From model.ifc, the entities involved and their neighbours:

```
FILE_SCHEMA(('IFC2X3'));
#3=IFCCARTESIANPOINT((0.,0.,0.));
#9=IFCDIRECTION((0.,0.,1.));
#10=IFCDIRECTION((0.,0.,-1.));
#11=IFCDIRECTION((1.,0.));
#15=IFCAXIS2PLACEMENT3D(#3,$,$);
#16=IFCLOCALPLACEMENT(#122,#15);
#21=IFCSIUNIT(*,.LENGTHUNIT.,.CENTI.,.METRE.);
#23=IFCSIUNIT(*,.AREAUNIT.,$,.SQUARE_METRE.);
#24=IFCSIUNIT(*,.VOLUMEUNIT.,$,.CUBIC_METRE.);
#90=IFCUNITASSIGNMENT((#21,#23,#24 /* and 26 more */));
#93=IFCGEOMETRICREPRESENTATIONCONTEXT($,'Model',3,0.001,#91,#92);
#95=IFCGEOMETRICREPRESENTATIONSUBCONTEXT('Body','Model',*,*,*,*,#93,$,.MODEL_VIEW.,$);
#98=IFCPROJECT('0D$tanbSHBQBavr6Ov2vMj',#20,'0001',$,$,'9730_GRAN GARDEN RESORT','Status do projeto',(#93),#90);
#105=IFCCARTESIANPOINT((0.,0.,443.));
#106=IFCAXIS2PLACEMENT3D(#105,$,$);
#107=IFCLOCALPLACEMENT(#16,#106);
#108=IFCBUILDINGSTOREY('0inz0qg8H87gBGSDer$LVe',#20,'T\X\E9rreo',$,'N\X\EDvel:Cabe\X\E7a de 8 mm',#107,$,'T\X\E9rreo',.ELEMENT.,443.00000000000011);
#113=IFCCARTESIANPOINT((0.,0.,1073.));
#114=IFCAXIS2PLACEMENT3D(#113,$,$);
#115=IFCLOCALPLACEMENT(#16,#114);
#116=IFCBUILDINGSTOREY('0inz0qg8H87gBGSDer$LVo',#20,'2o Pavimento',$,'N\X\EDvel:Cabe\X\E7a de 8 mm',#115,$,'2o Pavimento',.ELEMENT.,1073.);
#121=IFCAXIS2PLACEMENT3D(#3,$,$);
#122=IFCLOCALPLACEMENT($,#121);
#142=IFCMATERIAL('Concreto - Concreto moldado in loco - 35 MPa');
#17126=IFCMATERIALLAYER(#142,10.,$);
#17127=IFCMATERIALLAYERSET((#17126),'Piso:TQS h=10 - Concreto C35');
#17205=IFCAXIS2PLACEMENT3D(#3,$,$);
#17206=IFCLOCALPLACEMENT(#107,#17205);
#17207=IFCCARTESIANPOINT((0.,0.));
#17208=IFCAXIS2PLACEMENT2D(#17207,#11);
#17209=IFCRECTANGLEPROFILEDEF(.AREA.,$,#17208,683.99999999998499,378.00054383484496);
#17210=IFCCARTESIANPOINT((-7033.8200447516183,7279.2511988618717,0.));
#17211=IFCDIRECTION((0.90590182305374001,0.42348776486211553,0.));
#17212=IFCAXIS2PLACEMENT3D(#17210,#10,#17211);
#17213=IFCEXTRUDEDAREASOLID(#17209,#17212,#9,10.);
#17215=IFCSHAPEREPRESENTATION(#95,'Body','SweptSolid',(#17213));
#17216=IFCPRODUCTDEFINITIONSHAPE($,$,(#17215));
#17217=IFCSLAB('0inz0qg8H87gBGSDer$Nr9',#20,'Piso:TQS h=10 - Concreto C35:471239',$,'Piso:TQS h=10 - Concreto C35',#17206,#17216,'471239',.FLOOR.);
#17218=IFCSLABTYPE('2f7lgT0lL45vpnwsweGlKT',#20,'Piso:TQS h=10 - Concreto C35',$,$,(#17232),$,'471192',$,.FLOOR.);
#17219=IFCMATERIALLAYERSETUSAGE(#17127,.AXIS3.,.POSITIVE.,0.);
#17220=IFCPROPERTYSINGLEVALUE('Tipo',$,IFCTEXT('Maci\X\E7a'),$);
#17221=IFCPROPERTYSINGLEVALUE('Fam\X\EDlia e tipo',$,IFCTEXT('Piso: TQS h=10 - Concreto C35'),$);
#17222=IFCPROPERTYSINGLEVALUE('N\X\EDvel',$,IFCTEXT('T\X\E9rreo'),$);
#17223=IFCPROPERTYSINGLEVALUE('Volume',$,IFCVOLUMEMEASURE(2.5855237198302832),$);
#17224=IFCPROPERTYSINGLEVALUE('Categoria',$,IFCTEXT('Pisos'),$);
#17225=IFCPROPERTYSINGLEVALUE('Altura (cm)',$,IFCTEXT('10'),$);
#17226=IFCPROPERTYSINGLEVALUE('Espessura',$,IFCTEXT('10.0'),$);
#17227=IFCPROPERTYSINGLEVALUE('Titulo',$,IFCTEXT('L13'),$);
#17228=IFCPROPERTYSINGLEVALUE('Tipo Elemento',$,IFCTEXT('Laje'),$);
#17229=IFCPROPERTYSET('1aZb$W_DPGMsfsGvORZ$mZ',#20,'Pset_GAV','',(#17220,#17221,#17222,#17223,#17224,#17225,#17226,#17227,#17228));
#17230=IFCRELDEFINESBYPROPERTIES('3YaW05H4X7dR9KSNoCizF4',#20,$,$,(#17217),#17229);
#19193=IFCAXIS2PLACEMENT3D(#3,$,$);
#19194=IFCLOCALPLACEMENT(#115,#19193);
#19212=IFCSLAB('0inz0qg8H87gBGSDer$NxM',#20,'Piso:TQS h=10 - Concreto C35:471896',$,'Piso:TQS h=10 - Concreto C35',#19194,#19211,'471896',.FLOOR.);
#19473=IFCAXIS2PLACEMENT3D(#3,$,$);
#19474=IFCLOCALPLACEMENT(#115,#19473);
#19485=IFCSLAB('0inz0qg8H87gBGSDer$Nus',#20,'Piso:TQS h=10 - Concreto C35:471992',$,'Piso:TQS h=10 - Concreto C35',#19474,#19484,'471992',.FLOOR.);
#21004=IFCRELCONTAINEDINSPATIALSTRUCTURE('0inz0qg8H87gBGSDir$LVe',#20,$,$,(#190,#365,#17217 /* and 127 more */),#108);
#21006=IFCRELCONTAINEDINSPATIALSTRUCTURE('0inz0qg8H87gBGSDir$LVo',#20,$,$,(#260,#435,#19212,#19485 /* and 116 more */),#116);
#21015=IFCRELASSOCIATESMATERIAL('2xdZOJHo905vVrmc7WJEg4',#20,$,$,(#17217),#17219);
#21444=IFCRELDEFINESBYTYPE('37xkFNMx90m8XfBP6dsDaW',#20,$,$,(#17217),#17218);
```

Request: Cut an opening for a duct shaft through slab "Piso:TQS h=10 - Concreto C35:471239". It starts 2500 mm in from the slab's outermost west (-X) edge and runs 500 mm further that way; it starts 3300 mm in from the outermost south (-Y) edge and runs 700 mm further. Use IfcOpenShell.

```python
import numpy as np
import ifcopenshell
import ifcopenshell.api.feature
import ifcopenshell.api.geometry
import ifcopenshell.api.pset
import ifcopenshell.api.root
import ifcopenshell.geom
import ifcopenshell.util.element
import ifcopenshell.util.placement
import ifcopenshell.util.representation
import ifcopenshell.util.shape
import ifcopenshell.util.unit

model = ifcopenshell.open("model.ifc")
unit_scale = ifcopenshell.util.unit.calculate_unit_scale(model)
volume_scale = ifcopenshell.util.unit.calculate_unit_scale(model, "VOLUMEUNIT")
settings = ifcopenshell.geom.settings()


def volume(element):
    """Net volume in cubic metres, openings subtracted."""
    shape = ifcopenshell.geom.create_shape(settings, element)
    return ifcopenshell.util.shape.get_volume(shape.geometry)


slab = model.by_guid("0inz0qg8H87gBGSDer$Nr9")
before = volume(slab)

# Extent in the slab's own axes, in metres. The edges named are its -X and -Y sides.
slab_shape = ifcopenshell.geom.create_shape(settings, slab)
vertices = ifcopenshell.util.shape.get_vertices(slab_shape.geometry)
x_min, y_min, bottom = vertices.min(axis=0)
top = vertices[:, 2].max()

opening = ifcopenshell.api.root.create_entity(model, ifc_class="IfcOpeningElement", name="Duct shaft opening")
context = ifcopenshell.util.representation.get_context(model, "Model", "Body", "MODEL_VIEW")
width, depth = 0.5, 0.7
outline = [(0.0, 0.0), (width, 0.0), (width, depth), (0.0, depth), (0.0, 0.0)]
# Overshoot both faces by 50 mm so the cut is clean.
shape = ifcopenshell.api.geometry.add_slab_representation(
    model, context=context, depth=top - bottom + 0.1, polyline=outline
)
ifcopenshell.api.geometry.assign_representation(model, product=opening, representation=shape)

matrix = ifcopenshell.util.placement.get_local_placement(slab.ObjectPlacement)
matrix[:, 3] = matrix @ np.append(np.array([x_min + 2.5, y_min + 3.3, bottom - 0.05]) / unit_scale, 1.0)
ifcopenshell.api.geometry.edit_object_placement(model, product=opening, matrix=matrix, is_si=False)
ifcopenshell.api.feature.add_feature(model, feature=opening, element=slab)

after = volume(slab)

# Update the slab's stored quantities.
pset = model.by_id(ifcopenshell.util.element.get_pset(slab, "Pset_GAV", should_inherit=False)["id"])
ifcopenshell.api.pset.edit_pset(model, pset=pset, properties={
    "Volume": model.create_entity("IfcVolumeMeasure", after / volume_scale),
})

print(f"slab volume {before:.3f} -> {after:.3f} m3")

model.write("model-out.ifc")
```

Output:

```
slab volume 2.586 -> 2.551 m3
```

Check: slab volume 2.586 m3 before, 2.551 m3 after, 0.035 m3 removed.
